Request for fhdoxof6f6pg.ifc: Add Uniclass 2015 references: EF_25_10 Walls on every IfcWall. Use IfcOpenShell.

First a look at what the model holds.

```python
import ifcopenshell

model = ifcopenshell.open("fhdoxof6f6pg.ifc")
print(model.schema)
print("classifications:", [c.Name for c in model.by_type("IfcClassification")])
for ifc_class in ("IfcDoor", "IfcRoof", "IfcStair", "IfcWall", "IfcWindow"):
    print(ifc_class, len(model.by_type(ifc_class)))
```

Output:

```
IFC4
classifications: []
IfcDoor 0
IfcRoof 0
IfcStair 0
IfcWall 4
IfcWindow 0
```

```python
import ifcopenshell
import ifcopenshell.api.classification

model = ifcopenshell.open("fhdoxof6f6pg.ifc")

system = ifcopenshell.api.classification.add_classification(model, classification="Uniclass 2015")

codes = {
    "IfcWall": ("EF_25_10", "Walls"),
}
for ifc_class, (code, name) in codes.items():
    products = model.by_type(ifc_class)
    ifcopenshell.api.classification.add_reference(
        model, products=products, classification=system, identification=code, name=name
    )
    print(code, len(products))

model.write("fhdoxof6f6pg_rev.ifc")
```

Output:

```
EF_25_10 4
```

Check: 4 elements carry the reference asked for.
